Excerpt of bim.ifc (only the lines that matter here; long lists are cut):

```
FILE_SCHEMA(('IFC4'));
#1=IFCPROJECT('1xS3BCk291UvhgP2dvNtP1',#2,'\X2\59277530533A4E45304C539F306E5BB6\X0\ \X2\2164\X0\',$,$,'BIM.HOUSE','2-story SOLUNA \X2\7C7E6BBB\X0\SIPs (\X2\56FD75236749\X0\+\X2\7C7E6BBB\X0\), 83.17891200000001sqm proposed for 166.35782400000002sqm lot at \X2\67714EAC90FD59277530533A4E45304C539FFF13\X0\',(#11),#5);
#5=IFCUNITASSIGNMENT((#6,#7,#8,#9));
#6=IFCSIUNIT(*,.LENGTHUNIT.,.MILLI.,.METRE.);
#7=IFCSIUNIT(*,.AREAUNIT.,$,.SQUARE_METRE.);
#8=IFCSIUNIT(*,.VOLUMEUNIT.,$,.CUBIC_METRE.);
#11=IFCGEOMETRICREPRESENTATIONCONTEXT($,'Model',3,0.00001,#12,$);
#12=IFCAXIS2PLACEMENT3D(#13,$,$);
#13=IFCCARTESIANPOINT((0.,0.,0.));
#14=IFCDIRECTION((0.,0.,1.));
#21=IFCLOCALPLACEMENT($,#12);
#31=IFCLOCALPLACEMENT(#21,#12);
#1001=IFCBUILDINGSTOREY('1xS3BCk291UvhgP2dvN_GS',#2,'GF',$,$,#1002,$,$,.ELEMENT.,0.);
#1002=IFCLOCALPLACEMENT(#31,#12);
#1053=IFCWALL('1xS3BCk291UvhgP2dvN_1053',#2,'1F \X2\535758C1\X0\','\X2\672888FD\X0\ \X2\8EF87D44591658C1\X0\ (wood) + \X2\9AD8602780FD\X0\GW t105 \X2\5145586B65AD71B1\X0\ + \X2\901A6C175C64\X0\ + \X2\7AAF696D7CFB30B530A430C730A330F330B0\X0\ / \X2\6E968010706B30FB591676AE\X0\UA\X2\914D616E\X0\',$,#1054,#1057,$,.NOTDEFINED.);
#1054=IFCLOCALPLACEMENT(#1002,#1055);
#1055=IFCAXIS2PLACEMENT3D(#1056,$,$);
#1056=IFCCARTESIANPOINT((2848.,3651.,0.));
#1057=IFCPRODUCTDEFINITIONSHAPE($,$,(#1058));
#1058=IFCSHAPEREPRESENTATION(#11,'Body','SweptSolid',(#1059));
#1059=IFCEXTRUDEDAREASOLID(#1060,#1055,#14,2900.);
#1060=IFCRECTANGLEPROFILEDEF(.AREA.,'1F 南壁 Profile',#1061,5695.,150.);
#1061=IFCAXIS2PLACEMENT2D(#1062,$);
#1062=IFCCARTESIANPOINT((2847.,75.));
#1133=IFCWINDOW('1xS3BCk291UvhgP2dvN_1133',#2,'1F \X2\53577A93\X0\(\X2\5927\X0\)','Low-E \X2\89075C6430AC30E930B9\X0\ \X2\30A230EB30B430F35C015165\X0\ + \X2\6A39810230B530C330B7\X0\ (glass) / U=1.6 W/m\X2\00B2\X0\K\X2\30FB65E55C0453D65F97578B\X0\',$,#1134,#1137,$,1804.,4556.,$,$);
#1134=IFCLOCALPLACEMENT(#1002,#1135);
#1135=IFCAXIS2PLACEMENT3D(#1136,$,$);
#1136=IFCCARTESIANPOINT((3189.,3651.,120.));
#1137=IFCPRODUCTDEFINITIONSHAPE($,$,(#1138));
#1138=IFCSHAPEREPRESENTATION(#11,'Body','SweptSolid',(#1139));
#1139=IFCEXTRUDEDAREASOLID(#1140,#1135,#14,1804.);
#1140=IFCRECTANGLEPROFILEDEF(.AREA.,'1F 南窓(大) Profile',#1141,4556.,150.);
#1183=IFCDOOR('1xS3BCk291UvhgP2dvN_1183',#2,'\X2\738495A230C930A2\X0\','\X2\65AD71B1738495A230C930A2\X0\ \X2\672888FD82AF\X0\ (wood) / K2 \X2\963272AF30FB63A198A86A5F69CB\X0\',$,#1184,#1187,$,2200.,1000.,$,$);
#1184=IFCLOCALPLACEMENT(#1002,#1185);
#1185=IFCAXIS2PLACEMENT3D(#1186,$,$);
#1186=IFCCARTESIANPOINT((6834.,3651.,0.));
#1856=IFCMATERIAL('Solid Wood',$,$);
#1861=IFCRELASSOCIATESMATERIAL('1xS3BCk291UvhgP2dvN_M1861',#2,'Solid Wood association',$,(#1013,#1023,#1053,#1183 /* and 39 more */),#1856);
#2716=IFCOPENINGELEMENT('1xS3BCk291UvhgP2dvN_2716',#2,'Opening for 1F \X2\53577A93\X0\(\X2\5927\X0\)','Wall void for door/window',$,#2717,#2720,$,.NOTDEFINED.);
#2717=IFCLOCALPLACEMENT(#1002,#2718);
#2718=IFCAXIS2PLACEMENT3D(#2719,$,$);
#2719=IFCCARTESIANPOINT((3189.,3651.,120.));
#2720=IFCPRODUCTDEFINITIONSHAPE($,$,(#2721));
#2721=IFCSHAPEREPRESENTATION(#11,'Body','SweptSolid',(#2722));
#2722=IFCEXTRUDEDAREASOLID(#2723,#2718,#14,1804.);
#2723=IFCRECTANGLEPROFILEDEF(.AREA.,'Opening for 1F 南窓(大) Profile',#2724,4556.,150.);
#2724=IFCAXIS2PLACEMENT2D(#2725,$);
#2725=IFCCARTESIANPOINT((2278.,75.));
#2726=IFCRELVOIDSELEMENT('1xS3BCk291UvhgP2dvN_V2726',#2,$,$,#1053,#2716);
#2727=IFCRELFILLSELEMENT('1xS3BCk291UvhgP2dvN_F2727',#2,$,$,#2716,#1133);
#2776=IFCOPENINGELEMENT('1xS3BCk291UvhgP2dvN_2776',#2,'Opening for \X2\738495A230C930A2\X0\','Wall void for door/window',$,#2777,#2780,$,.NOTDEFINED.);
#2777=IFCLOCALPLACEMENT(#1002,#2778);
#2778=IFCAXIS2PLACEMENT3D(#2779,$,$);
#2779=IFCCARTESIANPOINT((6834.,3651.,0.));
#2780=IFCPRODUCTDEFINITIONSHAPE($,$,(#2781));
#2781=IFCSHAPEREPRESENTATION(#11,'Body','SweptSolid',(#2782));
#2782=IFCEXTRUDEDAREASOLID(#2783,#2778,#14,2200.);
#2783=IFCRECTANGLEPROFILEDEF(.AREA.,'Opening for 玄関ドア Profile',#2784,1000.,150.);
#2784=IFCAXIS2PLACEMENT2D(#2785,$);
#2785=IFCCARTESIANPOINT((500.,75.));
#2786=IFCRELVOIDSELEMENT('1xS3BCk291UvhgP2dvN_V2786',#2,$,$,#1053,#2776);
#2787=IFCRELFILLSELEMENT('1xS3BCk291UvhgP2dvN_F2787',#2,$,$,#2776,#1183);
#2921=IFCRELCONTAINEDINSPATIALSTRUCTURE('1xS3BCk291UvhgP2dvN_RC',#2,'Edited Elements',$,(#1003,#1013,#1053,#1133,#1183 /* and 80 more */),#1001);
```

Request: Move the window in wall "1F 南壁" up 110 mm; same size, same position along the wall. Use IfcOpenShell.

```python
import numpy as np
import ifcopenshell
import ifcopenshell.api.geometry
import ifcopenshell.util.placement
import ifcopenshell.util.unit

model = ifcopenshell.open("bim.ifc")
unit_scale = ifcopenshell.util.unit.calculate_unit_scale(model)

window = model.by_guid("1xS3BCk291UvhgP2dvN_1133")
opening = window.FillsVoids[0].RelatingOpeningElement
dz = 110.0

shift = np.array([0.0, 0.0, dz])
# The window is not placed relative to its opening, so move both.
for product in (opening, window):
    matrix = ifcopenshell.util.placement.get_local_placement(product.ObjectPlacement)
    matrix[:3, 3] += shift
    ifcopenshell.api.geometry.edit_object_placement(model, product=product, matrix=matrix, is_si=False)

print(f"moved by {dz * unit_scale:+.3f} m")

model.write("bim_v2.ifc")
```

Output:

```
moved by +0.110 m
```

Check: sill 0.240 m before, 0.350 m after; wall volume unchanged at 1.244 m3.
